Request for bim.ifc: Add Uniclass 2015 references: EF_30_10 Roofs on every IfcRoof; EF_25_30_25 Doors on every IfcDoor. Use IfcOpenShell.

First a look at what the model holds.

```python
import ifcopenshell

model = ifcopenshell.open("bim.ifc")
print(model.schema)
print("classifications:", [c.Name for c in model.by_type("IfcClassification")])
for ifc_class in ("IfcDoor", "IfcRoof", "IfcStair", "IfcWall", "IfcWindow"):
    print(ifc_class, len(model.by_type(ifc_class)))
```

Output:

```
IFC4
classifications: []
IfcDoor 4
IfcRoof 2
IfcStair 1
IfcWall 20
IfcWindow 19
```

```python
import ifcopenshell
import ifcopenshell.api.classification

model = ifcopenshell.open("bim.ifc")

system = ifcopenshell.api.classification.add_classification(model, classification="Uniclass 2015")

codes = {
    "IfcRoof": ("EF_30_10", "Roofs"),
    "IfcDoor": ("EF_25_30_25", "Doors"),
}
for ifc_class, (code, name) in codes.items():
    products = model.by_type(ifc_class)
    ifcopenshell.api.classification.add_reference(
        model, products=products, classification=system, identification=code, name=name
    )
    print(code, len(products))

model.write("bim_rev.ifc")
```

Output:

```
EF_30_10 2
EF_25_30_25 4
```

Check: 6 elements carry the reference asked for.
